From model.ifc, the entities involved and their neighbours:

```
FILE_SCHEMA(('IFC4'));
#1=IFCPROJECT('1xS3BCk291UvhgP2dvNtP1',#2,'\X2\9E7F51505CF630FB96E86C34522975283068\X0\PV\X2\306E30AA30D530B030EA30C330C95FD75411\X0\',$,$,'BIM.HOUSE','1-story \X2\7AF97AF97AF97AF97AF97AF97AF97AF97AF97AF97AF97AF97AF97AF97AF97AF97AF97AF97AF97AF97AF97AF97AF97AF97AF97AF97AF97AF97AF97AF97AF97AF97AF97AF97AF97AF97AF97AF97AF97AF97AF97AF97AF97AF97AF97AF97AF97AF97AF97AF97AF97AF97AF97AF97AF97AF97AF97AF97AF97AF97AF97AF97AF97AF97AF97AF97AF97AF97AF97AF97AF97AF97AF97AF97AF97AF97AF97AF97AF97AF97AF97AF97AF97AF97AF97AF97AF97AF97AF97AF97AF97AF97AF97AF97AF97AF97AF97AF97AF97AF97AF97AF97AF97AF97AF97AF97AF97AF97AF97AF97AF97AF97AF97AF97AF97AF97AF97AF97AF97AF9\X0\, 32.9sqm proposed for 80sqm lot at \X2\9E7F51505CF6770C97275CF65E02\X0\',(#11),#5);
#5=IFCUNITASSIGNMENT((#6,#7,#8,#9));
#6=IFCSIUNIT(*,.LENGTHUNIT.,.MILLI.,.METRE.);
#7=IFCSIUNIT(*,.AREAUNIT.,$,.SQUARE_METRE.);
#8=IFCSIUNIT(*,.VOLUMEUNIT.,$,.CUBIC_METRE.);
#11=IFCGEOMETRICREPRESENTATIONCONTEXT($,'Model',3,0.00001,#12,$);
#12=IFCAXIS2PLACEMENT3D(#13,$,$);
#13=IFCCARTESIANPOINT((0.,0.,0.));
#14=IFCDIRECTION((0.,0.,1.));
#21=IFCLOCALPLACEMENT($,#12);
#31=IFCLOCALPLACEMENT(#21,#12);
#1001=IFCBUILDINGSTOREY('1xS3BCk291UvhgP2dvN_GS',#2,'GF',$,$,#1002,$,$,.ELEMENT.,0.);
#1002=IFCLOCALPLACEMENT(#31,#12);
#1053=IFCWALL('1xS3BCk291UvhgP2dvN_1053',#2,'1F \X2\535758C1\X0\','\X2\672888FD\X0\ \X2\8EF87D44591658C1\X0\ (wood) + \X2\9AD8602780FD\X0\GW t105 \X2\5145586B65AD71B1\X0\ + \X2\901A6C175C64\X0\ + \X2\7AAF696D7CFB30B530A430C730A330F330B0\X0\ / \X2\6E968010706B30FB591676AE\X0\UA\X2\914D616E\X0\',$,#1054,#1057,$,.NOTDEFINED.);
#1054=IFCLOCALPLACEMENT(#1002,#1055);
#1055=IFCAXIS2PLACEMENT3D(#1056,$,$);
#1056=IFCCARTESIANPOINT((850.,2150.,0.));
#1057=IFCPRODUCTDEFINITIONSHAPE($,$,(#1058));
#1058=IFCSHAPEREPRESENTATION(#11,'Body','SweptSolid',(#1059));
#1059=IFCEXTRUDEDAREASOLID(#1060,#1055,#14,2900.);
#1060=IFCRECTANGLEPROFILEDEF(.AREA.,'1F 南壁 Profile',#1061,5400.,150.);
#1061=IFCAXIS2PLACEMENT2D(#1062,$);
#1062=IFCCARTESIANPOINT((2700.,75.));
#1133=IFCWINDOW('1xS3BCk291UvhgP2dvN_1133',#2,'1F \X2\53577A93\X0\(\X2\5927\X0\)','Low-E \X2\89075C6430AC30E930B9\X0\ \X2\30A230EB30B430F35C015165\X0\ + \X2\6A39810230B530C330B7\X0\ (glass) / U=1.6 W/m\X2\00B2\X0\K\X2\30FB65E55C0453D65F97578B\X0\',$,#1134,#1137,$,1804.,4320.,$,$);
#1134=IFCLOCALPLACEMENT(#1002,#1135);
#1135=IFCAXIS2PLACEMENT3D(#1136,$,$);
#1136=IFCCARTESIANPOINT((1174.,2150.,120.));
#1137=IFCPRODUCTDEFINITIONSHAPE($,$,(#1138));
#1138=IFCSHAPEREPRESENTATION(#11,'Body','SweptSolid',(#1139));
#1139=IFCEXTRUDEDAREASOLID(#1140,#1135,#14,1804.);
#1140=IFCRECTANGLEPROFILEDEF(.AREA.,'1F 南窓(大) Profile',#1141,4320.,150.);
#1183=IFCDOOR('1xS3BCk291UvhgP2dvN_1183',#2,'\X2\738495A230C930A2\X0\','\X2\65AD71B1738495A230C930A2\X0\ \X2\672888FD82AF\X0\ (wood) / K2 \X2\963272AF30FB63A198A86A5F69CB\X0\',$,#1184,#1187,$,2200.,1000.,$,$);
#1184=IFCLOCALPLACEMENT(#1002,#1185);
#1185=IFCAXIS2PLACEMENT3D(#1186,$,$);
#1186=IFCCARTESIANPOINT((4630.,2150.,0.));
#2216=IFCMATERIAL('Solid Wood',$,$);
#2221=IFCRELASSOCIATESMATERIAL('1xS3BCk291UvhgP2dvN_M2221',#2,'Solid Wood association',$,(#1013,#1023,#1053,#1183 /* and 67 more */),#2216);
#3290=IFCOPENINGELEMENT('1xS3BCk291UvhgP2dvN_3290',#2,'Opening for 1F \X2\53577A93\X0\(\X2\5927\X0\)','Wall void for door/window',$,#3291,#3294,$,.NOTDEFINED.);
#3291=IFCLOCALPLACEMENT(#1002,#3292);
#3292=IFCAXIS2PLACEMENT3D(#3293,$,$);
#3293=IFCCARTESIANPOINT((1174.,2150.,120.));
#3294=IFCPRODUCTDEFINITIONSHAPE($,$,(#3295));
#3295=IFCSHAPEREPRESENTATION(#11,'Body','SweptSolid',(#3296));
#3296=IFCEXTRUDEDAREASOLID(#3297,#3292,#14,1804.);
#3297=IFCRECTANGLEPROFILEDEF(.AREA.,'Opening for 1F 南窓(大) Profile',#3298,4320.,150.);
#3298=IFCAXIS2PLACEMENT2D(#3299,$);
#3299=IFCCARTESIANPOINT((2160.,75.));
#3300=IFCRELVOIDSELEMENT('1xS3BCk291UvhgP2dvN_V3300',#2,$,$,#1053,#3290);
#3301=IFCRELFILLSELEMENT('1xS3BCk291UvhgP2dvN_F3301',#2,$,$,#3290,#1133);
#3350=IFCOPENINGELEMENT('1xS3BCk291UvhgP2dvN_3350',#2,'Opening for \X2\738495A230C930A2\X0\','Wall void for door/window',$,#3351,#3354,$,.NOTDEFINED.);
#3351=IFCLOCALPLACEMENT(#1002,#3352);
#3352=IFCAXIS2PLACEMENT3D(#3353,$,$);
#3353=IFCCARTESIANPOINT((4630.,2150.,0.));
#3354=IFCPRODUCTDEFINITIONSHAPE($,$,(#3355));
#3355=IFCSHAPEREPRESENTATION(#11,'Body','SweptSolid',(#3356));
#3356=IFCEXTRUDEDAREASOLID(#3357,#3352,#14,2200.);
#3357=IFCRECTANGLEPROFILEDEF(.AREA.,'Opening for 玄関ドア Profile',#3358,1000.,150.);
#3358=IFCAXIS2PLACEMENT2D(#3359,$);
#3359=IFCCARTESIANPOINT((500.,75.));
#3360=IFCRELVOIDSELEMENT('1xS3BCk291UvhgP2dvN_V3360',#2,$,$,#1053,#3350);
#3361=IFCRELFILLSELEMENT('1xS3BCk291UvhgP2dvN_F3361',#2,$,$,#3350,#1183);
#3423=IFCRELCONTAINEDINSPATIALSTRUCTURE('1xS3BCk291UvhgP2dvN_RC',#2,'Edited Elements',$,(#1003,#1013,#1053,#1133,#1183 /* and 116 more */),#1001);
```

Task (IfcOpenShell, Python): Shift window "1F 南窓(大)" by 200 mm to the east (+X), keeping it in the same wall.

```python
import ifcopenshell
import ifcopenshell.api.geometry
import ifcopenshell.util.placement

model = ifcopenshell.open("model.ifc")

window = model.by_guid("1xS3BCk291UvhgP2dvN_1133")
opening = window.FillsVoids[0].RelatingOpeningElement
wall = opening.VoidsElements[0].RelatingBuildingElement

wall_matrix = ifcopenshell.util.placement.get_local_placement(wall.ObjectPlacement)
shift = wall_matrix[:3, 0] * 200.0
before = ifcopenshell.util.placement.get_local_placement(window.ObjectPlacement)[:3, 3].copy()

# The window is not placed relative to its opening, so move both.
for product in (opening, window):
    matrix = ifcopenshell.util.placement.get_local_placement(product.ObjectPlacement)
    matrix[:3, 3] += shift
    ifcopenshell.api.geometry.edit_object_placement(model, product=product, matrix=matrix, is_si=False)

after = ifcopenshell.util.placement.get_local_placement(window.ObjectPlacement)[:3, 3]
print("window moved by", (after - before).round(3) + 0.0)

model.write("model_rev.ifc")
```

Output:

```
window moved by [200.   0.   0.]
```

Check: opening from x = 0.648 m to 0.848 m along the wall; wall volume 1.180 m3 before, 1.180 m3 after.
